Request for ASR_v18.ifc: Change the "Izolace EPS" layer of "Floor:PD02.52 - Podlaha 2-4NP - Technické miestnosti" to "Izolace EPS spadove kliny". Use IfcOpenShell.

First a look at what the model holds.

```python
import ifcopenshell
import ifcopenshell.util.element

model = ifcopenshell.open("ASR_v18.ifc")
print(model.schema)
for layer_set in model.by_type("IfcMaterialLayerSet"):
    if layer_set.LayerSetName == "Floor:PD02.52 - Podlaha 2-4NP - Technické miestnosti":
        for layer in layer_set.MaterialLayers:
            print(layer.id(), layer.Material and layer.Material.Name, layer.LayerThickness, sep=" | ")
        print(len(ifcopenshell.util.element.get_elements_by_material(model, layer_set)), "elements and types use it")
print(sorted(m.Name for m in model.by_type("IfcMaterial") if m.Name)[:60])
```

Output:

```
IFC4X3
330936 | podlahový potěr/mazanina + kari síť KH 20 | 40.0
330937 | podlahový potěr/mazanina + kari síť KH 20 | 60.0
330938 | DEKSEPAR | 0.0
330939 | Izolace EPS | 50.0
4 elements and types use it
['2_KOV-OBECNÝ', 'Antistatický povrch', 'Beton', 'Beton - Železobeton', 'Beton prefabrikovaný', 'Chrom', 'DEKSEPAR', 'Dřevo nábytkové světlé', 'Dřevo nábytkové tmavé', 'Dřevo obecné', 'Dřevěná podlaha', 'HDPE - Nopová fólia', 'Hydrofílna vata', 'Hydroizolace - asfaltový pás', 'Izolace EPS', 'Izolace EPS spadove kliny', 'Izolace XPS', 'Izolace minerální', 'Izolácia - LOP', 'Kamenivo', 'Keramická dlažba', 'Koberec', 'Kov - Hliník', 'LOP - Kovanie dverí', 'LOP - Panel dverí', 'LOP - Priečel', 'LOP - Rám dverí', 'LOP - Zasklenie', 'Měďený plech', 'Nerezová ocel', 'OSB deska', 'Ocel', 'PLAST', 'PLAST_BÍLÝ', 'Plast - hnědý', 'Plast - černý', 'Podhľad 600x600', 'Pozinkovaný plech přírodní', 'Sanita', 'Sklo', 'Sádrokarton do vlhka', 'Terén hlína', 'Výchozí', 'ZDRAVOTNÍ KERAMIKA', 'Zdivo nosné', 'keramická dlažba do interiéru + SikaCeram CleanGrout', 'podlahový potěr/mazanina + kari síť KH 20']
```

```python
import ifcopenshell
import ifcopenshell.api.material

model = ifcopenshell.open("ASR_v18.ifc")

layer_set = next(s for s in model.by_type("IfcMaterialLayerSet") if s.LayerSetName == "Floor:PD02.52 - Podlaha 2-4NP - Technické miestnosti")
layer = next(l for l in layer_set.MaterialLayers if l.Material and l.Material.Name == "Izolace EPS")
material = next(m for m in model.by_type("IfcMaterial") if m.Name == "Izolace EPS spadove kliny")

# Point this one layer at the other material; renaming the old one would change it everywhere.
ifcopenshell.api.material.edit_layer(model, layer=layer, attributes={"Name": material.Name}, material=material)

print([l.Material.Name if l.Material else None for l in layer_set.MaterialLayers])

model.write("ASR_v18_v2.ifc")
```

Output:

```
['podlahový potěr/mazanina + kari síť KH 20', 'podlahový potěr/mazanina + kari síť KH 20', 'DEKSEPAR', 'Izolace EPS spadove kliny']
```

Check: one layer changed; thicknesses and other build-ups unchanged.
